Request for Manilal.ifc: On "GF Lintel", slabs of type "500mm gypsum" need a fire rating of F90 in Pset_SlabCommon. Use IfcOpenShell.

First a look at what the model holds.

```python
import ifcopenshell
import ifcopenshell.util.element

model = ifcopenshell.open("Manilal.ifc")
print(model.schema)
storey = next(s for s in model.by_type("IfcBuildingStorey") if s.Name == "GF Lintel")
slabs = [e for e in ifcopenshell.util.element.get_decomposition(storey) if e.is_a("IfcSlab")]
seen = {}
for e in slabs:
    element_type = ifcopenshell.util.element.get_type(e)
    key = (element_type.Name if element_type != e and element_type else None, ifcopenshell.util.element.get_pset(e, "Pset_SlabCommon", "FireRating"))
    seen[key] = seen.get(key, 0) + 1
for (name, value), count in sorted(seen.items(), key=str):
    print(count, "x", name, "|", value)
```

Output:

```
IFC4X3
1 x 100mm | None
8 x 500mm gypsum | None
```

```python
import ifcopenshell
import ifcopenshell.api.pset
import ifcopenshell.util.element

model = ifcopenshell.open("Manilal.ifc")

storey = next(s for s in model.by_type("IfcBuildingStorey") if s.Name == "GF Lintel")
slabs = [e for e in ifcopenshell.util.element.get_decomposition(storey) if e.is_a("IfcSlab")]

count = 0
for e in slabs:
    element_type = ifcopenshell.util.element.get_type(e)
    if element_type in (None, e) or element_type.Name != "500mm gypsum":
        continue
    # add_pset returns the element's existing set when there is one.
    pset = ifcopenshell.api.pset.add_pset(model, product=e, name="Pset_SlabCommon")
    ifcopenshell.api.pset.edit_pset(model, pset=pset, properties={"FireRating": "F90"})
    count += 1

print(count, "slabs updated")

model.write("Manilal_rev.ifc")
```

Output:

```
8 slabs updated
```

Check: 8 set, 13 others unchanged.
